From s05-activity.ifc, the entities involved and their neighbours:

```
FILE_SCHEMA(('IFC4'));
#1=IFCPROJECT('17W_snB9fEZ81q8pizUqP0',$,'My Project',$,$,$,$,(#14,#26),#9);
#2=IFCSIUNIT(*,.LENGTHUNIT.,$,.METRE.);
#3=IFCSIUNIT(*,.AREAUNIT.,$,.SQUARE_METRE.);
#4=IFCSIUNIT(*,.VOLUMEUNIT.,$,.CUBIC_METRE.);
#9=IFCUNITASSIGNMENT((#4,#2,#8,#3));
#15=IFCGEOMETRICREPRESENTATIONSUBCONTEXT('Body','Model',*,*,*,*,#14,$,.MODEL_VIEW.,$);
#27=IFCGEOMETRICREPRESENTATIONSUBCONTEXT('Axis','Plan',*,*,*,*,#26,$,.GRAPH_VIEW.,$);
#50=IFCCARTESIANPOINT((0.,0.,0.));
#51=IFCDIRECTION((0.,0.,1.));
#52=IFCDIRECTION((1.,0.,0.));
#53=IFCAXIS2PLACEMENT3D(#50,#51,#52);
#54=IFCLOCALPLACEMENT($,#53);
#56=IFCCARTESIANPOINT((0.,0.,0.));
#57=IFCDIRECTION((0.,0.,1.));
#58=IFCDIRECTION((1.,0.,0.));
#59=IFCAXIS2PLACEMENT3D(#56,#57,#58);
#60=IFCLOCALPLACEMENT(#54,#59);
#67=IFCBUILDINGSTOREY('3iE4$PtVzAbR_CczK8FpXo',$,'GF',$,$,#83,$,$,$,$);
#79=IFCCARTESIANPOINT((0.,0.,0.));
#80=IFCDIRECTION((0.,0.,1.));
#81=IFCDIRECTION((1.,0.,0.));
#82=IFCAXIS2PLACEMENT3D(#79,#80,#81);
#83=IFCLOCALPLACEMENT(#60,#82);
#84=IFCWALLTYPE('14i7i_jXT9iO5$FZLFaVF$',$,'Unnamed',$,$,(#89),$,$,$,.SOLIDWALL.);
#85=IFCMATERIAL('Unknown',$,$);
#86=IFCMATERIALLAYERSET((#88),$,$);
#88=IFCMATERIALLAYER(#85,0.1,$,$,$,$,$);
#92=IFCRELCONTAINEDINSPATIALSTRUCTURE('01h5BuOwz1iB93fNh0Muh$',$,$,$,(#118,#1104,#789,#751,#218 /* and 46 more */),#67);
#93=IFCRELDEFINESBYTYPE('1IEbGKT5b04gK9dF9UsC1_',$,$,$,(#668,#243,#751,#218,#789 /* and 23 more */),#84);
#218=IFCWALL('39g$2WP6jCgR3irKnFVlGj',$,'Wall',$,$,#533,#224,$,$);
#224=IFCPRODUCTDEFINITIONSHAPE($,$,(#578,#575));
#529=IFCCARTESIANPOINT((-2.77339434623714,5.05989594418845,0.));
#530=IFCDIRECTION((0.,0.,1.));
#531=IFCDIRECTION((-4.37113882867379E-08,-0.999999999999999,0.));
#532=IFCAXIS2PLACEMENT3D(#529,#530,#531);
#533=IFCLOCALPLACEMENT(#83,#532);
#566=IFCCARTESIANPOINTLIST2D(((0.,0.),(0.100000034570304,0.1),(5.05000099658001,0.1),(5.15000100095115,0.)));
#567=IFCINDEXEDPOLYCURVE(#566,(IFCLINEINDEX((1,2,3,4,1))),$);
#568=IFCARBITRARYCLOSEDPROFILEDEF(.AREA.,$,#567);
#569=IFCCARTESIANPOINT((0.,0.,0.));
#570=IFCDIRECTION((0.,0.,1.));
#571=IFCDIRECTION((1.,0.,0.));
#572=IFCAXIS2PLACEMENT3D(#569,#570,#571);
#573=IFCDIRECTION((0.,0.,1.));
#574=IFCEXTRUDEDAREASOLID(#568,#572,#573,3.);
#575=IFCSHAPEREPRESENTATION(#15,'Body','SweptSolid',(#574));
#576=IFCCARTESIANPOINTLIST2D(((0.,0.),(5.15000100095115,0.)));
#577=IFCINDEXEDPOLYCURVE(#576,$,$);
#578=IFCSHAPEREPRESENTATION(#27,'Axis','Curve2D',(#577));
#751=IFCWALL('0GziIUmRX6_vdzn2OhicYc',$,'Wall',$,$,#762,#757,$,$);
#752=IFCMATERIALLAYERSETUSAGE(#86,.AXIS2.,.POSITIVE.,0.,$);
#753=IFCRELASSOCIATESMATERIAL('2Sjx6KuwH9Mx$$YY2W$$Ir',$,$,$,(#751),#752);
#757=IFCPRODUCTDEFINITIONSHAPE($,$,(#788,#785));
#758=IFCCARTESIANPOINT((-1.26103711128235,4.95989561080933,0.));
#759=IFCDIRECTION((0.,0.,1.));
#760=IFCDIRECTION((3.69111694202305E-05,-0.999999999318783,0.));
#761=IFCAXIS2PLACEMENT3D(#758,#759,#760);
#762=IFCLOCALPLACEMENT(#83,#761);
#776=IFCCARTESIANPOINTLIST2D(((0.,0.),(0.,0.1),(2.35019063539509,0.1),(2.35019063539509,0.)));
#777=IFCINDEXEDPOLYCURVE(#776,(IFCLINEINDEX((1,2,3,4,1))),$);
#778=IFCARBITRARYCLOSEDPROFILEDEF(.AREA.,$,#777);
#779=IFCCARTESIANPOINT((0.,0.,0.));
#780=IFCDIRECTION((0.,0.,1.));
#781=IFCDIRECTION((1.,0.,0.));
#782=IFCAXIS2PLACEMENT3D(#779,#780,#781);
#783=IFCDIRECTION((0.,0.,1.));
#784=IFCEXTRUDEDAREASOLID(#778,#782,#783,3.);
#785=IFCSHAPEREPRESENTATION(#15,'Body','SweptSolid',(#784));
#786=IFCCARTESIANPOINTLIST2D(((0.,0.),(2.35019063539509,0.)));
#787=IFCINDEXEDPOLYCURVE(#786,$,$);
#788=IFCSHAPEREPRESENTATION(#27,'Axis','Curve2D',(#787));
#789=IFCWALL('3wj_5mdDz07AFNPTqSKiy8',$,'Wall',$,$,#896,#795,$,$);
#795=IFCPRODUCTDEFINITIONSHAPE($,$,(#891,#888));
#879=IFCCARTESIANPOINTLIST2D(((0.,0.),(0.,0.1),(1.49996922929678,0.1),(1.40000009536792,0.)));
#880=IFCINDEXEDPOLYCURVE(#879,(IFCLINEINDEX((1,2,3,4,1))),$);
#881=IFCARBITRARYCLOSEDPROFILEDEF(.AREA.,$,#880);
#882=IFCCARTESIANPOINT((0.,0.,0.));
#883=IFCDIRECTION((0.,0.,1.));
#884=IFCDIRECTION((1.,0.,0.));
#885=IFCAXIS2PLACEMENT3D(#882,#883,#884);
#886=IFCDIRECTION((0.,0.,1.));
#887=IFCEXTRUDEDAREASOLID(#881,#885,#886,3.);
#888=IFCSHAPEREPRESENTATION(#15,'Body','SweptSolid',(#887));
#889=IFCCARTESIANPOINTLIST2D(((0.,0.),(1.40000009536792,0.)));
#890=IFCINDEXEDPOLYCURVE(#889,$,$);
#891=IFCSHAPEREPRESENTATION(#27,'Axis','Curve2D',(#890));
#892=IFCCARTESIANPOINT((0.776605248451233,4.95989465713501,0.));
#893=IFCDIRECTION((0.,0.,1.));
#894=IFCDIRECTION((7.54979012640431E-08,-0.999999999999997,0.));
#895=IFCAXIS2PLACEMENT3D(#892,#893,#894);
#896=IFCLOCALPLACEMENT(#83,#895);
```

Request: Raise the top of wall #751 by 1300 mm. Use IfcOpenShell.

```python
import ifcopenshell
import ifcopenshell.geom
import ifcopenshell.util.representation
import ifcopenshell.util.shape
import ifcopenshell.util.unit

model = ifcopenshell.open("s05-activity.ifc")
unit_scale = ifcopenshell.util.unit.calculate_unit_scale(model)
settings = ifcopenshell.geom.settings()


def volume(element):
    """Net volume in cubic metres, openings subtracted."""
    shape = ifcopenshell.geom.create_shape(settings, element)
    return ifcopenshell.util.shape.get_volume(shape.geometry)


wall = model.by_guid("0GziIUmRX6_vdzn2OhicYc")
before = volume(wall)

body = ifcopenshell.util.representation.get_representation(wall, "Model", "Body")
solid = body.Items[0]
old_height = solid.Depth
solid.Depth += 1.3 / unit_scale
after = volume(wall)

print(f"height {old_height:g} -> {solid.Depth:g}, volume {before:.3f} -> {after:.3f} m3")

model.write("s05-activity_rev.ifc")
```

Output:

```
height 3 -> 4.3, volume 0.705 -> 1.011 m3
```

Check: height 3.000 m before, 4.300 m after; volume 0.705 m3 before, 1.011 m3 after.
